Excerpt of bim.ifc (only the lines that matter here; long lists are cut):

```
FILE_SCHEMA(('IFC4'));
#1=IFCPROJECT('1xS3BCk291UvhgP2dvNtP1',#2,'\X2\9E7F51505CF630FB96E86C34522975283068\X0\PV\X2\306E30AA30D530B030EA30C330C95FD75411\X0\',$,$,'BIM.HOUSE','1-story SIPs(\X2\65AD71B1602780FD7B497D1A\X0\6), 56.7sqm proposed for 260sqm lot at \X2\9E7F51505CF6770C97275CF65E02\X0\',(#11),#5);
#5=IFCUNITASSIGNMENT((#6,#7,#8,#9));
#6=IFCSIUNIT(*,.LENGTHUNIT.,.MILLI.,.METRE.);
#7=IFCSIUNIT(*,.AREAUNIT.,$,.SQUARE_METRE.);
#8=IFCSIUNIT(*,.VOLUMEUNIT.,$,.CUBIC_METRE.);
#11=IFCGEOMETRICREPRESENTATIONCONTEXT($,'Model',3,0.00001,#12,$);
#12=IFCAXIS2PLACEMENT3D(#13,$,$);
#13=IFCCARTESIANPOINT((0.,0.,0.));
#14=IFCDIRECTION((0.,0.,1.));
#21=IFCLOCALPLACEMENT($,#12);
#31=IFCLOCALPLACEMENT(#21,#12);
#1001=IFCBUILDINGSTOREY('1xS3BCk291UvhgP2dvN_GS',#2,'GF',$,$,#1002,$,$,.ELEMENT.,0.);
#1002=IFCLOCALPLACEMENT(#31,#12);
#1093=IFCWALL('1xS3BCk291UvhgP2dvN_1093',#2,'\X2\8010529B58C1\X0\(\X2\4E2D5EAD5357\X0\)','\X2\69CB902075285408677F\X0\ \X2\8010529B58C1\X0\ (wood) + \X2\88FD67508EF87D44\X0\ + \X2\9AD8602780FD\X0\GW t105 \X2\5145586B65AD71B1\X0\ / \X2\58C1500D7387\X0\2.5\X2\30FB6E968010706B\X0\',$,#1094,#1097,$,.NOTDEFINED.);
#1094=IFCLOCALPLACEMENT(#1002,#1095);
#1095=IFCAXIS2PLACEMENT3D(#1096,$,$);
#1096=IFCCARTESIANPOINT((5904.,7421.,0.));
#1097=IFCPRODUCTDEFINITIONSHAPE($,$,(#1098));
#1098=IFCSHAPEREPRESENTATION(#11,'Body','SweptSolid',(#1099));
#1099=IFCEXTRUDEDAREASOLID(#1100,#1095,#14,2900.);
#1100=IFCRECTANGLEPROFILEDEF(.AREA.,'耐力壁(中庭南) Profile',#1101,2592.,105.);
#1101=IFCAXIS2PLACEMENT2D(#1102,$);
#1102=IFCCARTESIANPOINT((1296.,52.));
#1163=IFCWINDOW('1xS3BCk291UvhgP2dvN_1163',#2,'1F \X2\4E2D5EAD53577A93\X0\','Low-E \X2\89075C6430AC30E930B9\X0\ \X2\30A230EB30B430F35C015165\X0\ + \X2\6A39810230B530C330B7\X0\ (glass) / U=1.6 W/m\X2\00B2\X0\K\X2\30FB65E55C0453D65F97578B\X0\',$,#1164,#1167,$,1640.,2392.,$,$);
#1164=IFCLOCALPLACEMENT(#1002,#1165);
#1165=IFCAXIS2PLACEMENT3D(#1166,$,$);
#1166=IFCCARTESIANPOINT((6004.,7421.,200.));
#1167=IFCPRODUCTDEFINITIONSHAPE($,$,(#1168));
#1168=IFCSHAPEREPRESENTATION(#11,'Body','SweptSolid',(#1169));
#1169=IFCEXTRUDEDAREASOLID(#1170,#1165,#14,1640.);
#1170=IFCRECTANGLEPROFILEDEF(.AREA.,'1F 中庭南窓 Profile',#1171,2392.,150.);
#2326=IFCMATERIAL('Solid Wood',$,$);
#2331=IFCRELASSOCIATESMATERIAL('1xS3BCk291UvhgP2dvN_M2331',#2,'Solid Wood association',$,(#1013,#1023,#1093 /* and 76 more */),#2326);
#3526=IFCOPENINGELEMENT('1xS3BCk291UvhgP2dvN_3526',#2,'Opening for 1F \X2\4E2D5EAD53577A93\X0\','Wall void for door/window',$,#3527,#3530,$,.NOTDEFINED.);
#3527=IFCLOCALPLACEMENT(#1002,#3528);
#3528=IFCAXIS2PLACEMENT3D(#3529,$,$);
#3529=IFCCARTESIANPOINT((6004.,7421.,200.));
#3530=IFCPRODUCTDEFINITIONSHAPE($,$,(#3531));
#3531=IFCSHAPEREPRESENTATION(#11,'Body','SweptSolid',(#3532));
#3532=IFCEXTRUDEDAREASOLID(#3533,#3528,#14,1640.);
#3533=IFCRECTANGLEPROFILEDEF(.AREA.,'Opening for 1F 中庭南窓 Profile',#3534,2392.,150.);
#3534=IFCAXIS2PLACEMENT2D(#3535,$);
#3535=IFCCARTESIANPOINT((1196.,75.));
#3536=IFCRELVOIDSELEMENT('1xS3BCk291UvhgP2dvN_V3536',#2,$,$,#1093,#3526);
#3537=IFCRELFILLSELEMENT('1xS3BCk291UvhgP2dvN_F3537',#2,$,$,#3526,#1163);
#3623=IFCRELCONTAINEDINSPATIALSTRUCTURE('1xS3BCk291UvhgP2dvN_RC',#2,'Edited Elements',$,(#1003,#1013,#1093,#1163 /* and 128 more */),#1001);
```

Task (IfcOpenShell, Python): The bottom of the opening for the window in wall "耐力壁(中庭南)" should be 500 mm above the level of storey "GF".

```python
import numpy as np
import ifcopenshell
import ifcopenshell.api.geometry
import ifcopenshell.geom
import ifcopenshell.util.element
import ifcopenshell.util.placement
import ifcopenshell.util.shape
import ifcopenshell.util.unit

model = ifcopenshell.open("bim.ifc")
unit_scale = ifcopenshell.util.unit.calculate_unit_scale(model)

window = model.by_guid("1xS3BCk291UvhgP2dvN_1163")
opening = window.FillsVoids[0].RelatingOpeningElement
storey = ifcopenshell.util.element.get_container(window, ifc_class="IfcBuildingStorey")
level = ifcopenshell.util.placement.get_local_placement(storey.ObjectPlacement)[2, 3]

# The opening's origin need not be at the sill, so measure its lowest point.
shape = ifcopenshell.geom.create_shape(ifcopenshell.geom.settings(), opening)
bottom = ifcopenshell.util.shape.get_shape_bottom_elevation(shape, shape.geometry) / unit_scale
dz = level + 0.5 / unit_scale - bottom

shift = np.array([0.0, 0.0, dz])
# The window is not placed relative to its opening, so move both.
for product in (opening, window):
    matrix = ifcopenshell.util.placement.get_local_placement(product.ObjectPlacement)
    matrix[:3, 3] += shift
    ifcopenshell.api.geometry.edit_object_placement(model, product=product, matrix=matrix, is_si=False)

print(f"moved by {dz * unit_scale:+.3f} m")

model.write("bim_rev.ifc")
```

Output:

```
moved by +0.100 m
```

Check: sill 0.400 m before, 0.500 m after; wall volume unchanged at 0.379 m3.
